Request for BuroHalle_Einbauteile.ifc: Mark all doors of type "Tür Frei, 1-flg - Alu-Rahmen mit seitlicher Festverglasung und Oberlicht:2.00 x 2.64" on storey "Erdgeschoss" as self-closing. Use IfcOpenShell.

First a look at what the model holds.

```python
import ifcopenshell
import ifcopenshell.util.element

model = ifcopenshell.open("BuroHalle_Einbauteile.ifc")
print(model.schema)
storey = next(s for s in model.by_type("IfcBuildingStorey") if s.Name == "Erdgeschoss")
doors = [e for e in ifcopenshell.util.element.get_decomposition(storey) if e.is_a("IfcDoor")]
seen = {}
for e in doors:
    element_type = ifcopenshell.util.element.get_type(e)
    key = (element_type.Name if element_type != e and element_type else None, ifcopenshell.util.element.get_pset(e, "Pset_DoorCommon", "SelfClosing"))
    seen[key] = seen.get(key, 0) + 1
for (name, value), count in sorted(seen.items(), key=str):
    print(count, "x", name, "|", value)
```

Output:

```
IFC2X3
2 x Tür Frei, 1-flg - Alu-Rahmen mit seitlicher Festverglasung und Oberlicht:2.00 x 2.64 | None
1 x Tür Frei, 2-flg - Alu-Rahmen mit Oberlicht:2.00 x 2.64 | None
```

```python
import ifcopenshell
import ifcopenshell.api.pset
import ifcopenshell.util.element

model = ifcopenshell.open("BuroHalle_Einbauteile.ifc")

storey = next(s for s in model.by_type("IfcBuildingStorey") if s.Name == "Erdgeschoss")
doors = [e for e in ifcopenshell.util.element.get_decomposition(storey) if e.is_a("IfcDoor")]

count = 0
for e in doors:
    element_type = ifcopenshell.util.element.get_type(e)
    if element_type in (None, e) or element_type.Name != "Tür Frei, 1-flg - Alu-Rahmen mit seitlicher Festverglasung und Oberlicht:2.00 x 2.64":
        continue
    # add_pset returns the element's existing set when there is one.
    pset = ifcopenshell.api.pset.add_pset(model, product=e, name="Pset_DoorCommon")
    ifcopenshell.api.pset.edit_pset(model, pset=pset, properties={"SelfClosing": True})
    count += 1

print(count, "doors updated")

model.write("BuroHalle_Einbauteile_v2.ifc")
```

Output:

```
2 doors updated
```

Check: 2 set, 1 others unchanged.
